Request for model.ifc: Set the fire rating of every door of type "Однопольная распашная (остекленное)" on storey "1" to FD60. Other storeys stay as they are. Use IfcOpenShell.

First a look at what the model holds.

```python
import ifcopenshell
import ifcopenshell.util.element

model = ifcopenshell.open("model.ifc")
print(model.schema)
storey = next(s for s in model.by_type("IfcBuildingStorey") if s.Name == "1")
doors = [e for e in ifcopenshell.util.element.get_decomposition(storey) if e.is_a("IfcDoor")]
seen = {}
for e in doors:
    element_type = ifcopenshell.util.element.get_type(e)
    key = (element_type.Name if element_type != e and element_type else None, ifcopenshell.util.element.get_pset(e, "Pset_DoorCommon", "FireRating"))
    seen[key] = seen.get(key, 0) + 1
for (name, value), count in sorted(seen.items(), key=str):
    print(count, "x", name, "|", value)
```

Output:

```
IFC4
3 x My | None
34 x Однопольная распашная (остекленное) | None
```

```python
import ifcopenshell
import ifcopenshell.api.pset
import ifcopenshell.util.element

model = ifcopenshell.open("model.ifc")

storey = next(s for s in model.by_type("IfcBuildingStorey") if s.Name == "1")
doors = [e for e in ifcopenshell.util.element.get_decomposition(storey) if e.is_a("IfcDoor")]

count = 0
for e in doors:
    element_type = ifcopenshell.util.element.get_type(e)
    if element_type in (None, e) or element_type.Name != "Однопольная распашная (остекленное)":
        continue
    # add_pset returns the element's existing set when there is one.
    pset = ifcopenshell.api.pset.add_pset(model, product=e, name="Pset_DoorCommon")
    ifcopenshell.api.pset.edit_pset(model, pset=pset, properties={"FireRating": "FD60"})
    count += 1

print(count, "doors updated")

model.write("model_edited.ifc")
```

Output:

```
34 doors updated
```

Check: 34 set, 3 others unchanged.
